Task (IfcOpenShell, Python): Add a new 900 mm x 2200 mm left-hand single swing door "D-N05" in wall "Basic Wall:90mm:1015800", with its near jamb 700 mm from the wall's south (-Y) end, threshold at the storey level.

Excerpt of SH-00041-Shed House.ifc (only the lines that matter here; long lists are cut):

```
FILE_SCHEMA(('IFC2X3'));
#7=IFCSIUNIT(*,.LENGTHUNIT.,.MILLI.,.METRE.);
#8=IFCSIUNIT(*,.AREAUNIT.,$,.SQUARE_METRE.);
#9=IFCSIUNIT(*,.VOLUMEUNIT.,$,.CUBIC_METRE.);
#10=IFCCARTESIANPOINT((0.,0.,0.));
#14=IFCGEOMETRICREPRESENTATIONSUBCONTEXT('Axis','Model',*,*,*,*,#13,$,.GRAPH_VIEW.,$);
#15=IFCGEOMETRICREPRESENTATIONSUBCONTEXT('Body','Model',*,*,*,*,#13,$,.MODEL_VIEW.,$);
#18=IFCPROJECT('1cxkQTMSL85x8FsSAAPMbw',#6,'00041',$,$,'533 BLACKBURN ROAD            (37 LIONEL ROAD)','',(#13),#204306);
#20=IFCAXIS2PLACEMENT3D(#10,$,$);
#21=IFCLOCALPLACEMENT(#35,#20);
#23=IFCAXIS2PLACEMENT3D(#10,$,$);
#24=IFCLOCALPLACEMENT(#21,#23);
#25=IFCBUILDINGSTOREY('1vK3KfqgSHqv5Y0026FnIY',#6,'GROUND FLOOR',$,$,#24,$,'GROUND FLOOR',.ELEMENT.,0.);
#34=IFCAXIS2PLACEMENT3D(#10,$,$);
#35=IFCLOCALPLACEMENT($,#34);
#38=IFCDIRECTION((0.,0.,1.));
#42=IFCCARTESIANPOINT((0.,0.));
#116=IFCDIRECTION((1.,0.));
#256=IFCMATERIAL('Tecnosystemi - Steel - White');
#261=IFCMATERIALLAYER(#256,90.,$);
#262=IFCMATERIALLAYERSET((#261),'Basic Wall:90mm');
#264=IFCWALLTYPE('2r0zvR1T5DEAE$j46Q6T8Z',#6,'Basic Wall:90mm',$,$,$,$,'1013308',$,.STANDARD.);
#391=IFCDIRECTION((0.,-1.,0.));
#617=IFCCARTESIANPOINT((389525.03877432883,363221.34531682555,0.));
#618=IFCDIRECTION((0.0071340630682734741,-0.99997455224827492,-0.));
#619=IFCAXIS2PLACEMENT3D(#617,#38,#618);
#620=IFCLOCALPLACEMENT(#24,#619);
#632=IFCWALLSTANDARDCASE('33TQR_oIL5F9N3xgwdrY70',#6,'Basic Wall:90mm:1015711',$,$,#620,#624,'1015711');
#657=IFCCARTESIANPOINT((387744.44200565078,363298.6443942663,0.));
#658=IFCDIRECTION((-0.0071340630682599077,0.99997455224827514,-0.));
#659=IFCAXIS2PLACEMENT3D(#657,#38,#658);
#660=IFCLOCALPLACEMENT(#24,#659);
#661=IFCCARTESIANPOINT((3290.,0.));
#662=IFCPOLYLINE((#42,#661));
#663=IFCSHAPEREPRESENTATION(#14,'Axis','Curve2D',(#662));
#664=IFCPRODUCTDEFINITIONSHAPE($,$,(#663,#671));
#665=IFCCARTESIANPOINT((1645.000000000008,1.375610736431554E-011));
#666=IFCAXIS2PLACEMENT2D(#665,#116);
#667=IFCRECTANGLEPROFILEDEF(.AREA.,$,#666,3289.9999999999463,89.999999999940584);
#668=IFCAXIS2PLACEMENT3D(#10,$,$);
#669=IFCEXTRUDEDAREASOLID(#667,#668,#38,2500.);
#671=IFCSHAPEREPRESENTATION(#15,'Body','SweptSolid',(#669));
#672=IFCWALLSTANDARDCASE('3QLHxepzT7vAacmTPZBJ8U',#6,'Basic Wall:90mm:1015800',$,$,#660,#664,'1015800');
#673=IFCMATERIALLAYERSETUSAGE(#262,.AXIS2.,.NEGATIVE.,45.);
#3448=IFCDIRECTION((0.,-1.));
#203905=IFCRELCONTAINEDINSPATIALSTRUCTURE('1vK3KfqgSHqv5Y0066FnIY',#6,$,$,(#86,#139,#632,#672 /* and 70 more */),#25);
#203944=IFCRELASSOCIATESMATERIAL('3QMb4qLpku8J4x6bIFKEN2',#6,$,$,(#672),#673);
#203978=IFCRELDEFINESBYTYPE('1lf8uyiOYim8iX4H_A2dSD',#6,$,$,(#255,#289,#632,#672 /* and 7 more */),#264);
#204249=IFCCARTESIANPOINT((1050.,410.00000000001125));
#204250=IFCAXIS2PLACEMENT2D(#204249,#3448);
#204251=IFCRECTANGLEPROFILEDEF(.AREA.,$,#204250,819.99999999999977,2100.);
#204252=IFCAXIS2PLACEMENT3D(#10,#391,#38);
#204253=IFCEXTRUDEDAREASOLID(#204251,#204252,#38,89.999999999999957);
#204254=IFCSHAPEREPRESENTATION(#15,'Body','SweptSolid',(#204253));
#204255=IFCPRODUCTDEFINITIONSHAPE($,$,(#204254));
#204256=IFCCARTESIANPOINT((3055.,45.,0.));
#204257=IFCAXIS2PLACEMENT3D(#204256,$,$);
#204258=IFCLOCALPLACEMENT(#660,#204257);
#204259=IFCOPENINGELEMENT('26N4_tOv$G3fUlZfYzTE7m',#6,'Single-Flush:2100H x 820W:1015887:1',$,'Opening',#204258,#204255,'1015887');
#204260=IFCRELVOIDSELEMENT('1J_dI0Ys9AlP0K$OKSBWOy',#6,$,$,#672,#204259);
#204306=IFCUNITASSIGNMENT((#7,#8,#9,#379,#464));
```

```python
import numpy as np
import ifcopenshell
import ifcopenshell.api.feature
import ifcopenshell.api.geometry
import ifcopenshell.api.root
import ifcopenshell.api.spatial
import ifcopenshell.api.type
import ifcopenshell.geom
import ifcopenshell.util.element
import ifcopenshell.util.placement
import ifcopenshell.util.representation
import ifcopenshell.util.shape
import ifcopenshell.util.unit

model = ifcopenshell.open("SH-00041-Shed House.ifc")
unit_scale = ifcopenshell.util.unit.calculate_unit_scale(model)
settings = ifcopenshell.geom.settings()


def volume(element):
    """Net volume in cubic metres, openings subtracted."""
    shape = ifcopenshell.geom.create_shape(settings, element)
    return ifcopenshell.util.shape.get_volume(shape.geometry)


wall = model.by_guid("3QLHxepzT7vAacmTPZBJ8U")
storey = ifcopenshell.util.element.get_container(wall, ifc_class="IfcBuildingStorey")
context = ifcopenshell.util.representation.get_context(model, "Model", "Body", "MODEL_VIEW")
before = volume(wall)

width, height, from_end, sill = 0.9, 2.2, 0.7, 0.0  # metres

# The wall runs along its own X axis, and the end named is its -X end.
wall_shape = ifcopenshell.geom.create_shape(settings, wall)
x, y, z = ifcopenshell.util.shape.get_vertices(wall_shape.geometry).T
start = x.min() + from_end
face, thickness = float(y.min()), float(y.max() - y.min())
wall_matrix = ifcopenshell.util.placement.get_local_placement(wall.ObjectPlacement)
level = ifcopenshell.util.placement.get_local_placement(storey.ObjectPlacement)[2, 3]


def in_wall(x, y):
    """Placement at x, y metres in the wall's axes, at sill height."""
    matrix = wall_matrix.copy()
    matrix[:, 3] = wall_matrix @ np.array([x / unit_scale, y / unit_scale, 0.0, 1.0])
    matrix[2, 3] = level + sill / unit_scale
    return matrix


# Opening: a box that overshoots both wall faces by 50 mm.
opening = ifcopenshell.api.root.create_entity(model, ifc_class="IfcOpeningElement")
box = ifcopenshell.api.geometry.add_wall_representation(
    model, context=context, length=width, height=height, thickness=thickness + 0.1
)
ifcopenshell.api.geometry.assign_representation(model, product=opening, representation=box)
ifcopenshell.api.geometry.edit_object_placement(model, product=opening, matrix=in_wall(start, face - 0.05), is_si=False)
ifcopenshell.api.feature.add_feature(model, feature=opening, element=wall)

door = ifcopenshell.api.root.create_entity(model, ifc_class="IfcDoor", name="D-N05")
door.OverallWidth, door.OverallHeight = width / unit_scale, height / unit_scale
body = ifcopenshell.api.geometry.add_door_representation(
    model,
    context=context,
    overall_width=door.OverallWidth,
    overall_height=door.OverallHeight,
    operation_type="SINGLE_SWING_LEFT",
    lining_properties={"LiningDepth": thickness / unit_scale, "ThresholdDepth": thickness / unit_scale},
)
ifcopenshell.api.geometry.assign_representation(model, product=door, representation=body)
ifcopenshell.api.spatial.assign_container(model, products=[door], relating_structure=storey)
fills = ifcopenshell.api.feature.add_filling(model, opening=opening, element=door)
fills.OwnerHistory = door.OwnerHistory  # required in IFC2X3

# IFC2X3 keeps the operation on the door style.
style = ifcopenshell.api.root.create_entity(model, ifc_class="IfcDoorStyle", name="D-N05")
style.OperationType, style.ConstructionType = "SINGLE_SWING_LEFT", "NOTDEFINED"
style.ParameterTakesPrecedence = style.Sizeable = False
ifcopenshell.api.type.assign_type(model, related_objects=[door], relating_type=style)

# The lining spans the wall, so the door starts at the wall face.
ifcopenshell.api.geometry.edit_object_placement(model, product=door, matrix=in_wall(start, face), is_si=False)

after = volume(wall)

print(f"wall volume {before:.3f} -> {after:.3f} m3")

model.write("SH-00041-Shed House-out.ifc")
```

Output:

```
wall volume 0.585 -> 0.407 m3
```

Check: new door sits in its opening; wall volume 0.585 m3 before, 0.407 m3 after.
